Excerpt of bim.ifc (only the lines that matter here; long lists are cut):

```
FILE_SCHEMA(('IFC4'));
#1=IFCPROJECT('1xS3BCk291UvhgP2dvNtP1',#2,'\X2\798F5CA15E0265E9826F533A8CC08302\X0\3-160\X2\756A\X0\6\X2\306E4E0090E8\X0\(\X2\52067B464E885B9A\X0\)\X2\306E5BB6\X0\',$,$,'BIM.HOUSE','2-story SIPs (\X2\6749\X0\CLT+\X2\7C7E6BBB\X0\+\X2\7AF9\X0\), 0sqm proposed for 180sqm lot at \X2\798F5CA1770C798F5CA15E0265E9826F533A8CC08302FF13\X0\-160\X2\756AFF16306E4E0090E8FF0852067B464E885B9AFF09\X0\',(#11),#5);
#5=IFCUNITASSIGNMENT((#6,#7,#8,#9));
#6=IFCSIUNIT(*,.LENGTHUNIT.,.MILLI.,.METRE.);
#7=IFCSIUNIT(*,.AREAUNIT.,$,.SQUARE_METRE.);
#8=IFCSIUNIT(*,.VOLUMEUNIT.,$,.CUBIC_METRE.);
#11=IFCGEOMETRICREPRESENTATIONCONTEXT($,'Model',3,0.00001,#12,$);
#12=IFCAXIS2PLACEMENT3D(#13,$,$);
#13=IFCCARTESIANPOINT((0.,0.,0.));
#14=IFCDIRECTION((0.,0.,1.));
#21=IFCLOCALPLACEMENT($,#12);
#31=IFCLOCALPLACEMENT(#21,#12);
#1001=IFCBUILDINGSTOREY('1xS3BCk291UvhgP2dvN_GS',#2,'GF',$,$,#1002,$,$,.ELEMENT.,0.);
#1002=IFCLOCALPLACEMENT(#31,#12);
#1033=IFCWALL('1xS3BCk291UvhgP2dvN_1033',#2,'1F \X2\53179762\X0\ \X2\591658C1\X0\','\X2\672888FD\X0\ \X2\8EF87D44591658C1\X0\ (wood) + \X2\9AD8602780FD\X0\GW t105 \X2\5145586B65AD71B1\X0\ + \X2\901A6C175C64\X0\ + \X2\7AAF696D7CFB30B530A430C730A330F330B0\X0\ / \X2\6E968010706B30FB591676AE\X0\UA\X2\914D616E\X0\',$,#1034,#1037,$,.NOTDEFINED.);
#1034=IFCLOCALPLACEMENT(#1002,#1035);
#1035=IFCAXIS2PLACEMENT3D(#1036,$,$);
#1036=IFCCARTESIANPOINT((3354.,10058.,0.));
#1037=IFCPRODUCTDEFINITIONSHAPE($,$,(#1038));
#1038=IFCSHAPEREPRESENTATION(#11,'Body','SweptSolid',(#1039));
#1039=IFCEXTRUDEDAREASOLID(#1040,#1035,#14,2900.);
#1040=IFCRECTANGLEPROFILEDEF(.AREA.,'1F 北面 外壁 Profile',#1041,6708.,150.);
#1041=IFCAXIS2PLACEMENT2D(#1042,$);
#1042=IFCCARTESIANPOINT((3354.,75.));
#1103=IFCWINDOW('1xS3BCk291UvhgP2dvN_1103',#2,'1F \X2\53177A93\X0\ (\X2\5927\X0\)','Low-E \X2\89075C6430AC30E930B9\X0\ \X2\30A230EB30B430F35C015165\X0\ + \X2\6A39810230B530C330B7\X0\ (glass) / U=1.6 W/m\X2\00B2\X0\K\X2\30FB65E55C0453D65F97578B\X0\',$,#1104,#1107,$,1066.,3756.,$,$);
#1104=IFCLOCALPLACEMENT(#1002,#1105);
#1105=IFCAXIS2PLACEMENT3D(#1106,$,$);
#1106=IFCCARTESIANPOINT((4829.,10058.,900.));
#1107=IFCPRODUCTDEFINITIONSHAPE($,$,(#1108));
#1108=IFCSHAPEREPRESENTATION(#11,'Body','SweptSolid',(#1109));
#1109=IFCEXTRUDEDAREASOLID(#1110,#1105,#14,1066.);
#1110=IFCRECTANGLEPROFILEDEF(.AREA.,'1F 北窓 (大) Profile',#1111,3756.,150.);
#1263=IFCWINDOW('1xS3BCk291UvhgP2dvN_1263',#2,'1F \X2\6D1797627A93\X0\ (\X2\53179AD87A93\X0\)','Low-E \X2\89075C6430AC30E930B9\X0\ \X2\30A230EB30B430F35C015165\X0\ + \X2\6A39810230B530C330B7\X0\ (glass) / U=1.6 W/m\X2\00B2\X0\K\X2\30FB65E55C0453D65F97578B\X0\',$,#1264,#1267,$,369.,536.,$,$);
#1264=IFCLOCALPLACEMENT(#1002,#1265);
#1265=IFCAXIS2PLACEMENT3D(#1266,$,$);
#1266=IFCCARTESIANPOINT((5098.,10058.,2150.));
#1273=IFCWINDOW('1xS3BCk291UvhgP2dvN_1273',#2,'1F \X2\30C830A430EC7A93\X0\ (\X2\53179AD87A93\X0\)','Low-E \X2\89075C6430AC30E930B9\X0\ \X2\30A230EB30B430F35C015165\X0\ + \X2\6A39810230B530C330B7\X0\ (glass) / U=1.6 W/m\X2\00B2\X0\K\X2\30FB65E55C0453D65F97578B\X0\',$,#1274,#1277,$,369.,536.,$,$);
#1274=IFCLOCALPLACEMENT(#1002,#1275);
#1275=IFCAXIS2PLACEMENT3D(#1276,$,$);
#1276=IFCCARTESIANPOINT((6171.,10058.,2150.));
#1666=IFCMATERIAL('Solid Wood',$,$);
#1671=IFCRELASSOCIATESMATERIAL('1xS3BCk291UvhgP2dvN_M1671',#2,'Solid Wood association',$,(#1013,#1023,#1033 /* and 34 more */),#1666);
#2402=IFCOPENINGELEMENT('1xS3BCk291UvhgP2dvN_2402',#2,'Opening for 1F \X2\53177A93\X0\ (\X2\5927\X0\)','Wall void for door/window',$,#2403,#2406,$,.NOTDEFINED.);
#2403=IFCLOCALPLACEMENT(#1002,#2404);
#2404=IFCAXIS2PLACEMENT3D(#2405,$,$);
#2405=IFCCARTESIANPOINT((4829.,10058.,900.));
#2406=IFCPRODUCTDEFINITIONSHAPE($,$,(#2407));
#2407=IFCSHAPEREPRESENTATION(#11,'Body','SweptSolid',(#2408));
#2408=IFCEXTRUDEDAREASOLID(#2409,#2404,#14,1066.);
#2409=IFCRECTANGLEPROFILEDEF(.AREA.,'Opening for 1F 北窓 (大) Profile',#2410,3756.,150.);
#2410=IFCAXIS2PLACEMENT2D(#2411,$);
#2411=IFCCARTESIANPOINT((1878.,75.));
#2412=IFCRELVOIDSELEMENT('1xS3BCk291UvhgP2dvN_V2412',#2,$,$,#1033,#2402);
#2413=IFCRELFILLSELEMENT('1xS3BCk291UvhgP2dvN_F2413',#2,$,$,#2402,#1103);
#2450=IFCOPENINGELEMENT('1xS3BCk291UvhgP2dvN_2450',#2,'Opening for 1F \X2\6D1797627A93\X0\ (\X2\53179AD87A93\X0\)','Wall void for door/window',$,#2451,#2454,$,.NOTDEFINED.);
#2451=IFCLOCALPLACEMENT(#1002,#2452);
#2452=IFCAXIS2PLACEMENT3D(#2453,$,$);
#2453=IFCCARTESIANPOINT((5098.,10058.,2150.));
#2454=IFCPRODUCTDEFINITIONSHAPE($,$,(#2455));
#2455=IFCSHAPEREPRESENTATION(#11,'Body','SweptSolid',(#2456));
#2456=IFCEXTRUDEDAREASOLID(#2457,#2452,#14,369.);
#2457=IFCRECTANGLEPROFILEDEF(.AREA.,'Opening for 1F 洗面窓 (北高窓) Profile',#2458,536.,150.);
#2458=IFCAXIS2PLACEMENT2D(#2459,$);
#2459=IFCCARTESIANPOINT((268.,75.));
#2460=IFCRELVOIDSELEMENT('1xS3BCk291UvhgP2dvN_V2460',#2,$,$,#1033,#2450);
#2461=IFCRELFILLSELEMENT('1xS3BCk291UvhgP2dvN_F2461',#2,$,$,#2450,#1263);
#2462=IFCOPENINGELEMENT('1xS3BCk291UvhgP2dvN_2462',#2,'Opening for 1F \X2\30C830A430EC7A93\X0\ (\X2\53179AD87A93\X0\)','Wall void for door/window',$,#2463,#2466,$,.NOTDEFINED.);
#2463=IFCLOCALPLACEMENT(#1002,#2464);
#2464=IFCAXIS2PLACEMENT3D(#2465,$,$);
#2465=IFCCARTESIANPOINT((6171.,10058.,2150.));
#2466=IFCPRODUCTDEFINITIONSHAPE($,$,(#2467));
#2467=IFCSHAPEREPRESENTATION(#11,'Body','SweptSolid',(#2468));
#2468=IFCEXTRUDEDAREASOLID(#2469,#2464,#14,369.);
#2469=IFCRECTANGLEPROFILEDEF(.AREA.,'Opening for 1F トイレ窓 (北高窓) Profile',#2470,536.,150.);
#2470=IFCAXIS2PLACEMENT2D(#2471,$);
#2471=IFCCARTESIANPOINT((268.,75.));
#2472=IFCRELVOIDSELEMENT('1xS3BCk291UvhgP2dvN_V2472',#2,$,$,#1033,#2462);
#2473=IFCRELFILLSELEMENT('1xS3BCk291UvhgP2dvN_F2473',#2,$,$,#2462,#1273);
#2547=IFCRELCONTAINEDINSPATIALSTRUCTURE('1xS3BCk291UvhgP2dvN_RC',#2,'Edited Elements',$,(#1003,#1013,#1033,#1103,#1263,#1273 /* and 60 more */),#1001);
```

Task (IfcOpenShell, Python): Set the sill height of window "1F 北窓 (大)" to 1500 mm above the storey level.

```python
import numpy as np
import ifcopenshell
import ifcopenshell.api.geometry
import ifcopenshell.geom
import ifcopenshell.util.element
import ifcopenshell.util.placement
import ifcopenshell.util.shape
import ifcopenshell.util.unit

model = ifcopenshell.open("bim.ifc")
unit_scale = ifcopenshell.util.unit.calculate_unit_scale(model)

window = model.by_guid("1xS3BCk291UvhgP2dvN_1103")
opening = window.FillsVoids[0].RelatingOpeningElement
storey = ifcopenshell.util.element.get_container(window, ifc_class="IfcBuildingStorey")
level = ifcopenshell.util.placement.get_local_placement(storey.ObjectPlacement)[2, 3]

# The opening's origin need not be at the sill, so measure its lowest point.
shape = ifcopenshell.geom.create_shape(ifcopenshell.geom.settings(), opening)
bottom = ifcopenshell.util.shape.get_shape_bottom_elevation(shape, shape.geometry) / unit_scale
dz = level + 1.5 / unit_scale - bottom

shift = np.array([0.0, 0.0, dz])
# The window is not placed relative to its opening, so move both.
for product in (opening, window):
    matrix = ifcopenshell.util.placement.get_local_placement(product.ObjectPlacement)
    matrix[:3, 3] += shift
    ifcopenshell.api.geometry.edit_object_placement(model, product=product, matrix=matrix, is_si=False)

print(f"moved by {dz * unit_scale:+.3f} m")

model.write("bim-out.ifc")
```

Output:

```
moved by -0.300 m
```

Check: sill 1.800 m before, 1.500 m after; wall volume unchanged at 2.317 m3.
